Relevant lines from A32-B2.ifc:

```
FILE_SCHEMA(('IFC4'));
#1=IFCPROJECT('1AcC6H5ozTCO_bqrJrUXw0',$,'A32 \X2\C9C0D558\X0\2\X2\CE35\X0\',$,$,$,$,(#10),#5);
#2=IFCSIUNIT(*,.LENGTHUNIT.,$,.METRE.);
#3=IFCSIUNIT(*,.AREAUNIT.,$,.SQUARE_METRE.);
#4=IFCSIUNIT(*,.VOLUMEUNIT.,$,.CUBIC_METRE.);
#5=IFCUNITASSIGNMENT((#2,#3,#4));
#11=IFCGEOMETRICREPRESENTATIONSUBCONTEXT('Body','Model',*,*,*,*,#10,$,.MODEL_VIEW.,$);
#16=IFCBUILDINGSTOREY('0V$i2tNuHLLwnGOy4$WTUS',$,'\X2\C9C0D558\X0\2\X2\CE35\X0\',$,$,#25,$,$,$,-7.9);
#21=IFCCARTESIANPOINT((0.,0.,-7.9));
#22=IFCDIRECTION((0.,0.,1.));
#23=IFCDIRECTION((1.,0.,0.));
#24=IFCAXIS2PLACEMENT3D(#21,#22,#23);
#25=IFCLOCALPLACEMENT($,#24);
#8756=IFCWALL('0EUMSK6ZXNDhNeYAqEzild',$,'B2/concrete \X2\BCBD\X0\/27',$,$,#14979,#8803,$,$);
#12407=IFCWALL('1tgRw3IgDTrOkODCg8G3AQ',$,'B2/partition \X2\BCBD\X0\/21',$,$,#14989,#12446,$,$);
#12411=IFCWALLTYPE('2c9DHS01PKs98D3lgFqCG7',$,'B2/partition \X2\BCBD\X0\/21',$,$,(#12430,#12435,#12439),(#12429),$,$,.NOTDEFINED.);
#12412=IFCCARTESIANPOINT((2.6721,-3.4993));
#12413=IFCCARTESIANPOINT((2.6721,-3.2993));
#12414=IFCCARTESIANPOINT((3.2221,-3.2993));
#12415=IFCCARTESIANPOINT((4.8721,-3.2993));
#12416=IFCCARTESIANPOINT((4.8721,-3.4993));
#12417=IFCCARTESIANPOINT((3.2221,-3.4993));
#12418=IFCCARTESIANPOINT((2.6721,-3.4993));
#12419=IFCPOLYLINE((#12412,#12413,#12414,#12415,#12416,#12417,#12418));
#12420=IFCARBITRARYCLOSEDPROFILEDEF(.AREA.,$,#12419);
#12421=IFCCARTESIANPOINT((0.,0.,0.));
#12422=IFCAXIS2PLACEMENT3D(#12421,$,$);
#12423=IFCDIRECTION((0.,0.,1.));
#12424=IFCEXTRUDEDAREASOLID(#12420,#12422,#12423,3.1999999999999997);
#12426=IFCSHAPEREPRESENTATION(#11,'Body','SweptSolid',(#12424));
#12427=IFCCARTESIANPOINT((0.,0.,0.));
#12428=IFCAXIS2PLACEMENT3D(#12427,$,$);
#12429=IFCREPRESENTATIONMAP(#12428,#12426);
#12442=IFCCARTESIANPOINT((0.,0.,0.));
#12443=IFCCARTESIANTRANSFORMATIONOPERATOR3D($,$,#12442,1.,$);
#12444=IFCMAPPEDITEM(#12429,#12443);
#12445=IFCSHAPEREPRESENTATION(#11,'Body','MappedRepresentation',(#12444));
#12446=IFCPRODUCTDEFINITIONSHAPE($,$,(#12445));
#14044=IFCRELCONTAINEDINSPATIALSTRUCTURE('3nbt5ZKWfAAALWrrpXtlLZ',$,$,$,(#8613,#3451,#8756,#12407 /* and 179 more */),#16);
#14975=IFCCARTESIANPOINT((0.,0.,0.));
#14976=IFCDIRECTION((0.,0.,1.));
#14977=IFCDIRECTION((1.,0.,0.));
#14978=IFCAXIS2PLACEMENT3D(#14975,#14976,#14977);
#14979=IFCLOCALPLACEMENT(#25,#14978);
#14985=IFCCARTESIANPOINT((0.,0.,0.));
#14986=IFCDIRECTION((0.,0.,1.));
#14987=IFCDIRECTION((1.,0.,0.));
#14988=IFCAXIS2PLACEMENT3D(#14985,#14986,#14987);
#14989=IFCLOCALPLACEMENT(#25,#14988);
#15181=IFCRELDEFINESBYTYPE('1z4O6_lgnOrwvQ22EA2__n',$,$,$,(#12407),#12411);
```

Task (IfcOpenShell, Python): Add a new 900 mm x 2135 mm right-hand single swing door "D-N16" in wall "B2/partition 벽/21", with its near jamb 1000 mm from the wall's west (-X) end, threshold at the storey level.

```python
import numpy as np
import ifcopenshell
import ifcopenshell.api.feature
import ifcopenshell.api.geometry
import ifcopenshell.api.root
import ifcopenshell.api.spatial
import ifcopenshell.geom
import ifcopenshell.util.element
import ifcopenshell.util.placement
import ifcopenshell.util.representation
import ifcopenshell.util.shape
import ifcopenshell.util.unit

model = ifcopenshell.open("A32-B2.ifc")
unit_scale = ifcopenshell.util.unit.calculate_unit_scale(model)
settings = ifcopenshell.geom.settings()


def volume(element):
    """Net volume in cubic metres, openings subtracted."""
    shape = ifcopenshell.geom.create_shape(settings, element)
    return ifcopenshell.util.shape.get_volume(shape.geometry)


wall = model.by_id(12407)
storey = ifcopenshell.util.element.get_container(wall, ifc_class="IfcBuildingStorey")
context = ifcopenshell.util.representation.get_context(model, "Model", "Body", "MODEL_VIEW")
before = volume(wall)

width, height, from_end, sill = 0.9, 2.135, 1, 0.0  # metres

# The wall runs along its own X axis, and the end named is its -X end.
wall_shape = ifcopenshell.geom.create_shape(settings, wall)
x, y, z = ifcopenshell.util.shape.get_vertices(wall_shape.geometry).T
start = x.min() + from_end
face, thickness = float(y.min()), float(y.max() - y.min())
wall_matrix = ifcopenshell.util.placement.get_local_placement(wall.ObjectPlacement)
level = ifcopenshell.util.placement.get_local_placement(storey.ObjectPlacement)[2, 3]


def in_wall(x, y):
    """Placement at x, y metres in the wall's axes, at sill height."""
    matrix = wall_matrix.copy()
    matrix[:, 3] = wall_matrix @ np.array([x / unit_scale, y / unit_scale, 0.0, 1.0])
    matrix[2, 3] = level + sill / unit_scale
    return matrix


# Opening: a box that overshoots both wall faces by 50 mm.
opening = ifcopenshell.api.root.create_entity(model, ifc_class="IfcOpeningElement", predefined_type="OPENING")
box = ifcopenshell.api.geometry.add_wall_representation(
    model, context=context, length=width, height=height, thickness=thickness + 0.1
)
ifcopenshell.api.geometry.assign_representation(model, product=opening, representation=box)
ifcopenshell.api.geometry.edit_object_placement(model, product=opening, matrix=in_wall(start, face - 0.05), is_si=False)
ifcopenshell.api.feature.add_feature(model, feature=opening, element=wall)

door = ifcopenshell.api.root.create_entity(model, ifc_class="IfcDoor", name="D-N16", predefined_type="DOOR")
door.OverallWidth, door.OverallHeight = width / unit_scale, height / unit_scale
door.OperationType = "SINGLE_SWING_RIGHT"
body = ifcopenshell.api.geometry.add_door_representation(
    model,
    context=context,
    overall_width=door.OverallWidth,
    overall_height=door.OverallHeight,
    operation_type="SINGLE_SWING_RIGHT",
    lining_properties={"LiningDepth": thickness / unit_scale, "ThresholdDepth": thickness / unit_scale},
)
ifcopenshell.api.geometry.assign_representation(model, product=door, representation=body)
ifcopenshell.api.spatial.assign_container(model, products=[door], relating_structure=storey)
ifcopenshell.api.feature.add_filling(model, opening=opening, element=door)

# The lining spans the wall, so the door starts at the wall face.
ifcopenshell.api.geometry.edit_object_placement(model, product=door, matrix=in_wall(start, face), is_si=False)

after = volume(wall)

print(f"wall volume {before:.3f} -> {after:.3f} m3")

model.write("A32-B2-out.ifc")
```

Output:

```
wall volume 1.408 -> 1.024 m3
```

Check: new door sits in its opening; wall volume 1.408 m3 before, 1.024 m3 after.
